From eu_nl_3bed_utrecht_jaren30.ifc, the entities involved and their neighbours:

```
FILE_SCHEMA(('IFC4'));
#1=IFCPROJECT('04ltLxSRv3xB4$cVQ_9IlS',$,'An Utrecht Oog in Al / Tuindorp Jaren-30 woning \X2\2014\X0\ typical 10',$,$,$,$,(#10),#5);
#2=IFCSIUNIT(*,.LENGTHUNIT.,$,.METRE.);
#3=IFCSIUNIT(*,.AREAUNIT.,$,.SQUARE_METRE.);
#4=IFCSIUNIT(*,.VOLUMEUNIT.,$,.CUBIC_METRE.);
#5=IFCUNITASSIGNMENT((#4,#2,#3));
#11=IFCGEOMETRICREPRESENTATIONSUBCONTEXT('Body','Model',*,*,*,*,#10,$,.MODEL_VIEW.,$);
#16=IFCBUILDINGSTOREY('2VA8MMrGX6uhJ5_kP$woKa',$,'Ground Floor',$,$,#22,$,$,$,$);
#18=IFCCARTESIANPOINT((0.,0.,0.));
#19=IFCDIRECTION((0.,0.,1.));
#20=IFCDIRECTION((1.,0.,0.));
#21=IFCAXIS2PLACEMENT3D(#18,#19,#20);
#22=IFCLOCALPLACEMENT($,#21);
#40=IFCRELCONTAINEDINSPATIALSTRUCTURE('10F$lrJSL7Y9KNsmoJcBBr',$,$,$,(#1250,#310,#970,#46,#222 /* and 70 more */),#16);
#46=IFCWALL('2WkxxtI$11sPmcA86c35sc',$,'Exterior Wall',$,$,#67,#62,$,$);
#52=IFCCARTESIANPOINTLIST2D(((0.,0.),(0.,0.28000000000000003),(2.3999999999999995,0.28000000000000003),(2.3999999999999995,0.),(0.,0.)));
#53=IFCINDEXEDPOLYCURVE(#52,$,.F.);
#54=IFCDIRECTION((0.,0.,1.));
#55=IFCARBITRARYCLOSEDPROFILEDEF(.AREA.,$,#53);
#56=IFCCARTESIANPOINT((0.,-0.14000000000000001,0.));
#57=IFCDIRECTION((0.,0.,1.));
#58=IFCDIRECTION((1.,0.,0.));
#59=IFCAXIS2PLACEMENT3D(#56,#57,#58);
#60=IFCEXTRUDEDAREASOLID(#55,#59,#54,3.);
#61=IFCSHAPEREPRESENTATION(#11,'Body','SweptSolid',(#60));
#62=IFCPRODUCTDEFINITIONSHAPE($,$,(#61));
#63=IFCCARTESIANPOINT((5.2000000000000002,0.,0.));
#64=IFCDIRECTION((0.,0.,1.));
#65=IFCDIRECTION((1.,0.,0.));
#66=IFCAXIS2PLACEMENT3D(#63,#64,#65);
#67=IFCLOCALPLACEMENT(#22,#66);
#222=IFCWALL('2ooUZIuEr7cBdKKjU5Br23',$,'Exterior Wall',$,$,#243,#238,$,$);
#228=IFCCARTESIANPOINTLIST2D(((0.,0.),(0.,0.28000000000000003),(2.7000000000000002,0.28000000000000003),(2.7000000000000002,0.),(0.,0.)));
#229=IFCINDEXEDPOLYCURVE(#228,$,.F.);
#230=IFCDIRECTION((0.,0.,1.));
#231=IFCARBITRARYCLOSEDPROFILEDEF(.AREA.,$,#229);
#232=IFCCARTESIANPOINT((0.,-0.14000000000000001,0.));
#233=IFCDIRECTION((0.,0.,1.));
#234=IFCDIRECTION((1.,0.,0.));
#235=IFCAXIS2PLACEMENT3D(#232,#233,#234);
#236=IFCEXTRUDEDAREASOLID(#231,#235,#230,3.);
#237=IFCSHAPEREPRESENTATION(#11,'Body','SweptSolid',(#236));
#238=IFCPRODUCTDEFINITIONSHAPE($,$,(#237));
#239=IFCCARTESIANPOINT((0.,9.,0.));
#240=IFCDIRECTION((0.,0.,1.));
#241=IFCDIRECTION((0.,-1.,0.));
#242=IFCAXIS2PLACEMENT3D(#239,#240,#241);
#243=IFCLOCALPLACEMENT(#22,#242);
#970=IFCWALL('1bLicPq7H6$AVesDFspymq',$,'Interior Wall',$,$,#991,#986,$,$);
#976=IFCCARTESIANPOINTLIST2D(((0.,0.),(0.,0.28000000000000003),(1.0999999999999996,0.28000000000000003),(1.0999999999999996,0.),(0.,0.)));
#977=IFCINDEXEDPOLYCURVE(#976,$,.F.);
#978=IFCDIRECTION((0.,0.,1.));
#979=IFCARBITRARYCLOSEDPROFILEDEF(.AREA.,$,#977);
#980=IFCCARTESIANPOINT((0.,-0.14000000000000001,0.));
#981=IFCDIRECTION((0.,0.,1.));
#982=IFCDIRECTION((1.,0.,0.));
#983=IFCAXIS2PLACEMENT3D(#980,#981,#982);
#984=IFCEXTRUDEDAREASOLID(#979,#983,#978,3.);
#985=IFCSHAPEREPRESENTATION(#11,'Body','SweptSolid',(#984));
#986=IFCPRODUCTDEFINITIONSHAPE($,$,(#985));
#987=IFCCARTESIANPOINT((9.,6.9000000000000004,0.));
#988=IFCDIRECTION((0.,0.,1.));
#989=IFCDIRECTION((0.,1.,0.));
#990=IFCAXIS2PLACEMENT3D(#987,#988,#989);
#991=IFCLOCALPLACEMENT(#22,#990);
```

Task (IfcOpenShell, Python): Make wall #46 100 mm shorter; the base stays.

```python
import ifcopenshell
import ifcopenshell.geom
import ifcopenshell.util.representation
import ifcopenshell.util.shape

model = ifcopenshell.open("eu_nl_3bed_utrecht_jaren30.ifc")
settings = ifcopenshell.geom.settings()


def volume(element):
    """Net volume in cubic metres, openings subtracted."""
    shape = ifcopenshell.geom.create_shape(settings, element)
    return ifcopenshell.util.shape.get_volume(shape.geometry)


wall = model.by_id(46)
before = volume(wall)

body = ifcopenshell.util.representation.get_representation(wall, "Model", "Body")
solid = body.Items[0]
old_height = solid.Depth
solid.Depth -= 0.1
after = volume(wall)

print(f"height {old_height:g} -> {solid.Depth:g}, volume {before:.3f} -> {after:.3f} m3")

model.write("eu_nl_3bed_utrecht_jaren30_edited.ifc")
```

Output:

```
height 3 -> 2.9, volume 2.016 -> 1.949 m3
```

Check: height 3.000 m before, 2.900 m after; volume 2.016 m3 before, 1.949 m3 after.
